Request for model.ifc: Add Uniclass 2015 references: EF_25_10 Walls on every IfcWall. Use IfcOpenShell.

First a look at what the model holds.

```python
import ifcopenshell

model = ifcopenshell.open("model.ifc")
print(model.schema)
print("classifications:", [c.Name for c in model.by_type("IfcClassification")])
for ifc_class in ("IfcDoor", "IfcRoof", "IfcStair", "IfcWall", "IfcWindow"):
    print(ifc_class, len(model.by_type(ifc_class)))
```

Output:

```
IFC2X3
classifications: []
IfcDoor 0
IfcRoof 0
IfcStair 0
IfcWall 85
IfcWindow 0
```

```python
import ifcopenshell
import ifcopenshell.api.classification

model = ifcopenshell.open("model.ifc")

# IFC2X3 requires Source and Edition and has no link from the project to the system.
system = model.create_entity("IfcClassification", Source="NBS", Edition="2015", Name="Uniclass 2015")

codes = {
    "IfcWall": ("EF_25_10", "Walls"),
}
for ifc_class, (code, name) in codes.items():
    products = model.by_type(ifc_class)
    ifcopenshell.api.classification.add_reference(
        model, products=products, classification=system, identification=code, name=name
    )
    print(code, len(products))

model.write("model_updated.ifc")
```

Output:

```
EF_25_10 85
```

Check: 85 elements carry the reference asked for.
